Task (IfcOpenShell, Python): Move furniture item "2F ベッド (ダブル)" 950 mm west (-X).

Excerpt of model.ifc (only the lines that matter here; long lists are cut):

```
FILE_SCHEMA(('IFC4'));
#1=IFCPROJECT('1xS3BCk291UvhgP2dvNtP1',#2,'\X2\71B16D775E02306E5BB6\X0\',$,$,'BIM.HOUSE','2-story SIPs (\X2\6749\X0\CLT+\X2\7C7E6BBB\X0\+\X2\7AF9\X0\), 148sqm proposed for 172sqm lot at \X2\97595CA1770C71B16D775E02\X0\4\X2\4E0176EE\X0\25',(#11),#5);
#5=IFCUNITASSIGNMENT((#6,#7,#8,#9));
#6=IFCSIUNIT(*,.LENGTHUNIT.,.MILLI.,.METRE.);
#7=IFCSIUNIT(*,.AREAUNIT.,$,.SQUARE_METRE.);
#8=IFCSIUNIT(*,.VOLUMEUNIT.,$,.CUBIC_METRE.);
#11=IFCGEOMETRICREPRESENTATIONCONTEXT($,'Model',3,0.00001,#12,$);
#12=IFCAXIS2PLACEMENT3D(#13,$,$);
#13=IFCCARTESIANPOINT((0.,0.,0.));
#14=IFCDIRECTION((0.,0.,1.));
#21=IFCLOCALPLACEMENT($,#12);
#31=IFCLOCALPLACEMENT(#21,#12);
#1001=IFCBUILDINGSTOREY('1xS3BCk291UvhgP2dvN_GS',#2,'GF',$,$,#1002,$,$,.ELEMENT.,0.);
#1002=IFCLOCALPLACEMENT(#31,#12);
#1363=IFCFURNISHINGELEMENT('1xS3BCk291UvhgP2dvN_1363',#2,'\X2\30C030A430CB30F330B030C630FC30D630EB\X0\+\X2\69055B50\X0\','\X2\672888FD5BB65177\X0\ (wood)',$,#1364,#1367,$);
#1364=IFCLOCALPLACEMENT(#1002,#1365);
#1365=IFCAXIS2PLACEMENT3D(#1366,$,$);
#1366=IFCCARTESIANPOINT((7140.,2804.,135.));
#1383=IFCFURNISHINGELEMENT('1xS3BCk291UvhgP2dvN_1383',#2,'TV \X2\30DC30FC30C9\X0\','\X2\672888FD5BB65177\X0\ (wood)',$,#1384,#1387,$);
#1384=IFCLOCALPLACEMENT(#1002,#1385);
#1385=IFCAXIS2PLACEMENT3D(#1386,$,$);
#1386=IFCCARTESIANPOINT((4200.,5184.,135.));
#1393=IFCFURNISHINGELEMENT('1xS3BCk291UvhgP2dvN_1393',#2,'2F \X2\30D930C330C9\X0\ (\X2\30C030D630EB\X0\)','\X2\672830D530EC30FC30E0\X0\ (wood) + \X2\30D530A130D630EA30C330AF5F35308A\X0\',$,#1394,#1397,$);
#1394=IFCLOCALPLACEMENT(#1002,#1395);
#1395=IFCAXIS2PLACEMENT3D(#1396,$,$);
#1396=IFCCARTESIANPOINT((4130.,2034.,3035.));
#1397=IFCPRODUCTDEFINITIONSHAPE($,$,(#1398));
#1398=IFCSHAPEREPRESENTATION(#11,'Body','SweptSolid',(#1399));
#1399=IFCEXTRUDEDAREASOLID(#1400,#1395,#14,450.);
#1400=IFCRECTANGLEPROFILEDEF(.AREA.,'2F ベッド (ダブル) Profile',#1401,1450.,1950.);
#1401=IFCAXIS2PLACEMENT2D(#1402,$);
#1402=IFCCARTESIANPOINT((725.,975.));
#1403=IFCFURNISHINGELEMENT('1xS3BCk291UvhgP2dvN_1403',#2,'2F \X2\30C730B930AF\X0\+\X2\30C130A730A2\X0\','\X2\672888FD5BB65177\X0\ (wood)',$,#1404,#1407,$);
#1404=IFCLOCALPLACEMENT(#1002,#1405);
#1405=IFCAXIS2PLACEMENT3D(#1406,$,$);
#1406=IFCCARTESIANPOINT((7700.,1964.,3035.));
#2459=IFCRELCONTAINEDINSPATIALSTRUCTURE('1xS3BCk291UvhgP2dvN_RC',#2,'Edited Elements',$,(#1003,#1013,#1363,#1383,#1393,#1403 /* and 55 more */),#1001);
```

```python
import ifcopenshell
import ifcopenshell.api.geometry
import ifcopenshell.util.placement
import ifcopenshell.util.unit

model = ifcopenshell.open("model.ifc")
unit_scale = ifcopenshell.util.unit.calculate_unit_scale(model)

item = model.by_guid("1xS3BCk291UvhgP2dvN_1393")
matrix = ifcopenshell.util.placement.get_local_placement(item.ObjectPlacement)
matrix[0, 3] -= 0.95 / unit_scale
ifcopenshell.api.geometry.edit_object_placement(model, product=item, matrix=matrix, is_si=False)

print(ifcopenshell.util.placement.get_local_placement(item.ObjectPlacement).round(3) + 0.0)

model.write("model_updated.ifc")
```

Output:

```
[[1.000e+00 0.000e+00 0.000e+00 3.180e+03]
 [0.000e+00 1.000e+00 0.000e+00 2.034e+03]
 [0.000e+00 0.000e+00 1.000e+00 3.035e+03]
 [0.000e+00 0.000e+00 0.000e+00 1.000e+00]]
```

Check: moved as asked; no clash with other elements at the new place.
